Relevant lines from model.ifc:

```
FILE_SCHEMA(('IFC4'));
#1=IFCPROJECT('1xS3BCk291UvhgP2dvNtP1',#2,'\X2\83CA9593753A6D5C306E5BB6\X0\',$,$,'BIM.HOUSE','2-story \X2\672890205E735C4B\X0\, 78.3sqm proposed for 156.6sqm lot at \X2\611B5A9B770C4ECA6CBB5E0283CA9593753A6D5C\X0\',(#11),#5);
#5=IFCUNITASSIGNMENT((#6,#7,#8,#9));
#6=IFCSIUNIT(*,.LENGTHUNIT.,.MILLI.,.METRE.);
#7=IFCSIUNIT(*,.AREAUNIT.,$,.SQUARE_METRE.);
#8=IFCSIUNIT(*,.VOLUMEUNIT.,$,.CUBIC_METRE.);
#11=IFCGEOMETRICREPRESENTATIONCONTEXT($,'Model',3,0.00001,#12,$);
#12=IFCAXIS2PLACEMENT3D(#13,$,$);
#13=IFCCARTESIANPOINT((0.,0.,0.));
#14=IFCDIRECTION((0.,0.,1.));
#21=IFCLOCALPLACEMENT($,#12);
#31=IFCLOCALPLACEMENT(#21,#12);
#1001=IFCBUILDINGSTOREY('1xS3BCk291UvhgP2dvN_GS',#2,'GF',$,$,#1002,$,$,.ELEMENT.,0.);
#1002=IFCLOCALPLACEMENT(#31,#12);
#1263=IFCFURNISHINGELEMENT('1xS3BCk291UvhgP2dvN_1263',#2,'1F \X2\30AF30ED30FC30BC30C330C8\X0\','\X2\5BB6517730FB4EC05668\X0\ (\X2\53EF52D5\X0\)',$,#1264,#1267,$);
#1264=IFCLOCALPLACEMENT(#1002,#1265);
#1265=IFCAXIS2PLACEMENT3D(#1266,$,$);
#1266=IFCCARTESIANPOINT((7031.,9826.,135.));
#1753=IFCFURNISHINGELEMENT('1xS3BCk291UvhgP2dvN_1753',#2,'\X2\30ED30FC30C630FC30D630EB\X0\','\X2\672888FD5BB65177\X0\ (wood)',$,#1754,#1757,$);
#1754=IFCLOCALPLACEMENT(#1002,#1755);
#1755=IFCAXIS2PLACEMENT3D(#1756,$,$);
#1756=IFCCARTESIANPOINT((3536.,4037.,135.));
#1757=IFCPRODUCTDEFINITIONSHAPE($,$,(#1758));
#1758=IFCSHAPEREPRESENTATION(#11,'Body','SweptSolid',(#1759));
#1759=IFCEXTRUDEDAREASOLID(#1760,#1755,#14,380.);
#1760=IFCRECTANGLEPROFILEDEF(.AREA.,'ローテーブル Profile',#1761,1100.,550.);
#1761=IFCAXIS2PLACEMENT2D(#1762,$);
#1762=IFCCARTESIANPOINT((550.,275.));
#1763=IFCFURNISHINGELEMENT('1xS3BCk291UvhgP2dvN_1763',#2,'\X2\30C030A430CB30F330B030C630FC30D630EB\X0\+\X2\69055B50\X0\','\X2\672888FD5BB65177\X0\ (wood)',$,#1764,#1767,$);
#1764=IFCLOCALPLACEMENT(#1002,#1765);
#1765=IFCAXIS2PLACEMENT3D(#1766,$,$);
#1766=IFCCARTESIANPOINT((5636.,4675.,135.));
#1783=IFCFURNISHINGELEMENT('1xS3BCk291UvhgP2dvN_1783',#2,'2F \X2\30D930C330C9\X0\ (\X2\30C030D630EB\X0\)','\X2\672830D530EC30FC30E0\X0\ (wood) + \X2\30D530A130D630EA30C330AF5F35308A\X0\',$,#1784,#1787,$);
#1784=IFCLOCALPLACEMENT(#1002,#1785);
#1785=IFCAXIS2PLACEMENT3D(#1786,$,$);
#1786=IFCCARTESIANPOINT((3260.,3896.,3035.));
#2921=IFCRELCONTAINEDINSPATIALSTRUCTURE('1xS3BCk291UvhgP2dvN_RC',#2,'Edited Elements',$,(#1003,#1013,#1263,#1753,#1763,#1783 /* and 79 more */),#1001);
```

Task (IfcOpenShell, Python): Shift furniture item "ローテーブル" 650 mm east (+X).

```python
import ifcopenshell
import ifcopenshell.api.geometry
import ifcopenshell.util.placement
import ifcopenshell.util.unit

model = ifcopenshell.open("model.ifc")
unit_scale = ifcopenshell.util.unit.calculate_unit_scale(model)

item = model.by_id(1753)
matrix = ifcopenshell.util.placement.get_local_placement(item.ObjectPlacement)
matrix[0, 3] += 0.65 / unit_scale
ifcopenshell.api.geometry.edit_object_placement(model, product=item, matrix=matrix, is_si=False)

print(ifcopenshell.util.placement.get_local_placement(item.ObjectPlacement).round(3) + 0.0)

model.write("model-out.ifc")
```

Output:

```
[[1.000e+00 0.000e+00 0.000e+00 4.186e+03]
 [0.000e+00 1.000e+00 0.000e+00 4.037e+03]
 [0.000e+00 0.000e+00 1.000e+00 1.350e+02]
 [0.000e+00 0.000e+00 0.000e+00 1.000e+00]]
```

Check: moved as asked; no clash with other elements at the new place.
